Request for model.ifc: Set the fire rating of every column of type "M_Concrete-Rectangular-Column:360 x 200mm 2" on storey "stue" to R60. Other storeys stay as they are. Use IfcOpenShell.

First a look at what the model holds.

```python
import ifcopenshell
import ifcopenshell.util.element

model = ifcopenshell.open("model.ifc")
print(model.schema)
storey = next(s for s in model.by_type("IfcBuildingStorey") if s.Name == "stue")
columns = [e for e in ifcopenshell.util.element.get_decomposition(storey) if e.is_a("IfcColumn")]
seen = {}
for e in columns:
    element_type = ifcopenshell.util.element.get_type(e)
    key = (element_type.Name if element_type != e and element_type else None, ifcopenshell.util.element.get_pset(e, "Pset_ColumnCommon", "FireRating"))
    seen[key] = seen.get(key, 0) + 1
for (name, value), count in sorted(seen.items(), key=str):
    print(count, "x", name, "|", value)
```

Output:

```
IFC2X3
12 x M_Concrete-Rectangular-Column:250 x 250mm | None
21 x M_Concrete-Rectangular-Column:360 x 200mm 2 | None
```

```python
import ifcopenshell
import ifcopenshell.api.pset
import ifcopenshell.util.element

model = ifcopenshell.open("model.ifc")

storey = next(s for s in model.by_type("IfcBuildingStorey") if s.Name == "stue")
columns = [e for e in ifcopenshell.util.element.get_decomposition(storey) if e.is_a("IfcColumn")]

count = 0
for e in columns:
    element_type = ifcopenshell.util.element.get_type(e)
    if element_type in (None, e) or element_type.Name != "M_Concrete-Rectangular-Column:360 x 200mm 2":
        continue
    # add_pset returns the element's existing set when there is one.
    pset = ifcopenshell.api.pset.add_pset(model, product=e, name="Pset_ColumnCommon")
    ifcopenshell.api.pset.edit_pset(model, pset=pset, properties={"FireRating": "R60"})
    count += 1

print(count, "columns updated")

model.write("model-out.ifc")
```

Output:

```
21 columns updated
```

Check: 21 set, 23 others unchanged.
